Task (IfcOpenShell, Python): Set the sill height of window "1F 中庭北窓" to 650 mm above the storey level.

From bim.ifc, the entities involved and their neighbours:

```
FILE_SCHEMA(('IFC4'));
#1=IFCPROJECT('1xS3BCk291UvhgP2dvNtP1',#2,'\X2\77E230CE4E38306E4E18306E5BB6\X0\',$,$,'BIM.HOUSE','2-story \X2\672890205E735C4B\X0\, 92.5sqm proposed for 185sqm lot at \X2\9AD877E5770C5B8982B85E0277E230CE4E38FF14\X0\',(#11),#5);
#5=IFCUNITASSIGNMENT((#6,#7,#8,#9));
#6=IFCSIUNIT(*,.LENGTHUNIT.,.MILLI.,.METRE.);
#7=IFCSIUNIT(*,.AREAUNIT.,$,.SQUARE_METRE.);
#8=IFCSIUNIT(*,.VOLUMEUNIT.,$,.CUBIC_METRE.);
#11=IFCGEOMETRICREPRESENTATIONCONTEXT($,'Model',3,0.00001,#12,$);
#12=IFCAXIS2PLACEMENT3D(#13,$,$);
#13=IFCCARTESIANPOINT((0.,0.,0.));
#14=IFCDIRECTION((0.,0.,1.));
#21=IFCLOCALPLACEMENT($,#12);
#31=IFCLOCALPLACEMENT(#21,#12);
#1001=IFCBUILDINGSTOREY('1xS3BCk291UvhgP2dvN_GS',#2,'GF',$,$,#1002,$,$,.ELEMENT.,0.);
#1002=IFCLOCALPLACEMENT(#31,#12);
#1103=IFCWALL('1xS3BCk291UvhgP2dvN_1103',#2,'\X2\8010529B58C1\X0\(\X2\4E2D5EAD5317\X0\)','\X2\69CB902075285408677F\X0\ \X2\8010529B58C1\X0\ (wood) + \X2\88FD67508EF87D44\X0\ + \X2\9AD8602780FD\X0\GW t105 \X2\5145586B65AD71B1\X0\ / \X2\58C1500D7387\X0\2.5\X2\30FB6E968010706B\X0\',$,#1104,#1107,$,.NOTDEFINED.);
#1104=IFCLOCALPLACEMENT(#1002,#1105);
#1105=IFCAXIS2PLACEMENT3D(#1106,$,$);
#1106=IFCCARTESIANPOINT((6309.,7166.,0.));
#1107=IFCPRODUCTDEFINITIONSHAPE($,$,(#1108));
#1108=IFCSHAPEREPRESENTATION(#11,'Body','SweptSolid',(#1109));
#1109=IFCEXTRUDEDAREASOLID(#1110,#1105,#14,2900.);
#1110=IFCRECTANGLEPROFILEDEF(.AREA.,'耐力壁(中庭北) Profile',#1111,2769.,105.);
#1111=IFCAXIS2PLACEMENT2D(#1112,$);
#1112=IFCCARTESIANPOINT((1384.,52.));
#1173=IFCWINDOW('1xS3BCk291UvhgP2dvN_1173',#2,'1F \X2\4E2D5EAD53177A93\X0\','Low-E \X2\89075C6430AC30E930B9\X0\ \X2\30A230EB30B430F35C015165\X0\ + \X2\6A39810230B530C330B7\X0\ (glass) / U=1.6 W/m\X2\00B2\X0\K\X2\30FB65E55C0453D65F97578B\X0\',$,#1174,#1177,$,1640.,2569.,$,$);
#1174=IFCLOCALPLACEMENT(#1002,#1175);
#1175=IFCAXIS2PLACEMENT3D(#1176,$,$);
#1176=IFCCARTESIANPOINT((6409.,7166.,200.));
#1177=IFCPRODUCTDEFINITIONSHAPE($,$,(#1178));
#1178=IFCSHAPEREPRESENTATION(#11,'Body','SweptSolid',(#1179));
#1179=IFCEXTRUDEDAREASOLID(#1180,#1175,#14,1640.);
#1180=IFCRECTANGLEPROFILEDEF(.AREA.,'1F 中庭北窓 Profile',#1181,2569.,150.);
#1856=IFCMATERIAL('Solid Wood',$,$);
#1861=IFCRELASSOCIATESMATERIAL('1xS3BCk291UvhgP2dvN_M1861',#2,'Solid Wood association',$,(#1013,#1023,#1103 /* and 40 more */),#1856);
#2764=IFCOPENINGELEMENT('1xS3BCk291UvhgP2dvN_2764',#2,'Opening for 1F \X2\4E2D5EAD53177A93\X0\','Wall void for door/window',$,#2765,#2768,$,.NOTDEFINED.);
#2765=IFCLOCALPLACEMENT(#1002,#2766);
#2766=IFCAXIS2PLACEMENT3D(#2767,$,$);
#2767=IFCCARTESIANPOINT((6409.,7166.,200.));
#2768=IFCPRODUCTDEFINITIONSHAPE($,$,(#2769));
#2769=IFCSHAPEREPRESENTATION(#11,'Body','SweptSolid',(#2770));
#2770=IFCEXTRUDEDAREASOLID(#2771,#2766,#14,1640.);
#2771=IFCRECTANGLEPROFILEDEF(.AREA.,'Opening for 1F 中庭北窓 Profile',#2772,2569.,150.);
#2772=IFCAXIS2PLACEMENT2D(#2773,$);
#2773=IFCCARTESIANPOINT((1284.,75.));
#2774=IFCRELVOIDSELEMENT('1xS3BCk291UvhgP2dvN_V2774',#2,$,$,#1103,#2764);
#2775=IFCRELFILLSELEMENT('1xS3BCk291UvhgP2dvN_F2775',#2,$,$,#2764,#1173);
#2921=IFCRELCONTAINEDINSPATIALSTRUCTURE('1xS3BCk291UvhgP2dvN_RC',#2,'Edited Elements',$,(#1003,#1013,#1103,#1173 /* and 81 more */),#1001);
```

```python
import numpy as np
import ifcopenshell
import ifcopenshell.api.geometry
import ifcopenshell.geom
import ifcopenshell.util.element
import ifcopenshell.util.placement
import ifcopenshell.util.shape
import ifcopenshell.util.unit

model = ifcopenshell.open("bim.ifc")
unit_scale = ifcopenshell.util.unit.calculate_unit_scale(model)

window = model.by_id(1173)
opening = window.FillsVoids[0].RelatingOpeningElement
storey = ifcopenshell.util.element.get_container(window, ifc_class="IfcBuildingStorey")
level = ifcopenshell.util.placement.get_local_placement(storey.ObjectPlacement)[2, 3]

# The opening's origin need not be at the sill, so measure its lowest point.
shape = ifcopenshell.geom.create_shape(ifcopenshell.geom.settings(), opening)
bottom = ifcopenshell.util.shape.get_shape_bottom_elevation(shape, shape.geometry) / unit_scale
dz = level + 0.65 / unit_scale - bottom

shift = np.array([0.0, 0.0, dz])
# The window is not placed relative to its opening, so move both.
for product in (opening, window):
    matrix = ifcopenshell.util.placement.get_local_placement(product.ObjectPlacement)
    matrix[:3, 3] += shift
    ifcopenshell.api.geometry.edit_object_placement(model, product=product, matrix=matrix, is_si=False)

print(f"moved by {dz * unit_scale:+.3f} m")

model.write("bim_updated.ifc")
```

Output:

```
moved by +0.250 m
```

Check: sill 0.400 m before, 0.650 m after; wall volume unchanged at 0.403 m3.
